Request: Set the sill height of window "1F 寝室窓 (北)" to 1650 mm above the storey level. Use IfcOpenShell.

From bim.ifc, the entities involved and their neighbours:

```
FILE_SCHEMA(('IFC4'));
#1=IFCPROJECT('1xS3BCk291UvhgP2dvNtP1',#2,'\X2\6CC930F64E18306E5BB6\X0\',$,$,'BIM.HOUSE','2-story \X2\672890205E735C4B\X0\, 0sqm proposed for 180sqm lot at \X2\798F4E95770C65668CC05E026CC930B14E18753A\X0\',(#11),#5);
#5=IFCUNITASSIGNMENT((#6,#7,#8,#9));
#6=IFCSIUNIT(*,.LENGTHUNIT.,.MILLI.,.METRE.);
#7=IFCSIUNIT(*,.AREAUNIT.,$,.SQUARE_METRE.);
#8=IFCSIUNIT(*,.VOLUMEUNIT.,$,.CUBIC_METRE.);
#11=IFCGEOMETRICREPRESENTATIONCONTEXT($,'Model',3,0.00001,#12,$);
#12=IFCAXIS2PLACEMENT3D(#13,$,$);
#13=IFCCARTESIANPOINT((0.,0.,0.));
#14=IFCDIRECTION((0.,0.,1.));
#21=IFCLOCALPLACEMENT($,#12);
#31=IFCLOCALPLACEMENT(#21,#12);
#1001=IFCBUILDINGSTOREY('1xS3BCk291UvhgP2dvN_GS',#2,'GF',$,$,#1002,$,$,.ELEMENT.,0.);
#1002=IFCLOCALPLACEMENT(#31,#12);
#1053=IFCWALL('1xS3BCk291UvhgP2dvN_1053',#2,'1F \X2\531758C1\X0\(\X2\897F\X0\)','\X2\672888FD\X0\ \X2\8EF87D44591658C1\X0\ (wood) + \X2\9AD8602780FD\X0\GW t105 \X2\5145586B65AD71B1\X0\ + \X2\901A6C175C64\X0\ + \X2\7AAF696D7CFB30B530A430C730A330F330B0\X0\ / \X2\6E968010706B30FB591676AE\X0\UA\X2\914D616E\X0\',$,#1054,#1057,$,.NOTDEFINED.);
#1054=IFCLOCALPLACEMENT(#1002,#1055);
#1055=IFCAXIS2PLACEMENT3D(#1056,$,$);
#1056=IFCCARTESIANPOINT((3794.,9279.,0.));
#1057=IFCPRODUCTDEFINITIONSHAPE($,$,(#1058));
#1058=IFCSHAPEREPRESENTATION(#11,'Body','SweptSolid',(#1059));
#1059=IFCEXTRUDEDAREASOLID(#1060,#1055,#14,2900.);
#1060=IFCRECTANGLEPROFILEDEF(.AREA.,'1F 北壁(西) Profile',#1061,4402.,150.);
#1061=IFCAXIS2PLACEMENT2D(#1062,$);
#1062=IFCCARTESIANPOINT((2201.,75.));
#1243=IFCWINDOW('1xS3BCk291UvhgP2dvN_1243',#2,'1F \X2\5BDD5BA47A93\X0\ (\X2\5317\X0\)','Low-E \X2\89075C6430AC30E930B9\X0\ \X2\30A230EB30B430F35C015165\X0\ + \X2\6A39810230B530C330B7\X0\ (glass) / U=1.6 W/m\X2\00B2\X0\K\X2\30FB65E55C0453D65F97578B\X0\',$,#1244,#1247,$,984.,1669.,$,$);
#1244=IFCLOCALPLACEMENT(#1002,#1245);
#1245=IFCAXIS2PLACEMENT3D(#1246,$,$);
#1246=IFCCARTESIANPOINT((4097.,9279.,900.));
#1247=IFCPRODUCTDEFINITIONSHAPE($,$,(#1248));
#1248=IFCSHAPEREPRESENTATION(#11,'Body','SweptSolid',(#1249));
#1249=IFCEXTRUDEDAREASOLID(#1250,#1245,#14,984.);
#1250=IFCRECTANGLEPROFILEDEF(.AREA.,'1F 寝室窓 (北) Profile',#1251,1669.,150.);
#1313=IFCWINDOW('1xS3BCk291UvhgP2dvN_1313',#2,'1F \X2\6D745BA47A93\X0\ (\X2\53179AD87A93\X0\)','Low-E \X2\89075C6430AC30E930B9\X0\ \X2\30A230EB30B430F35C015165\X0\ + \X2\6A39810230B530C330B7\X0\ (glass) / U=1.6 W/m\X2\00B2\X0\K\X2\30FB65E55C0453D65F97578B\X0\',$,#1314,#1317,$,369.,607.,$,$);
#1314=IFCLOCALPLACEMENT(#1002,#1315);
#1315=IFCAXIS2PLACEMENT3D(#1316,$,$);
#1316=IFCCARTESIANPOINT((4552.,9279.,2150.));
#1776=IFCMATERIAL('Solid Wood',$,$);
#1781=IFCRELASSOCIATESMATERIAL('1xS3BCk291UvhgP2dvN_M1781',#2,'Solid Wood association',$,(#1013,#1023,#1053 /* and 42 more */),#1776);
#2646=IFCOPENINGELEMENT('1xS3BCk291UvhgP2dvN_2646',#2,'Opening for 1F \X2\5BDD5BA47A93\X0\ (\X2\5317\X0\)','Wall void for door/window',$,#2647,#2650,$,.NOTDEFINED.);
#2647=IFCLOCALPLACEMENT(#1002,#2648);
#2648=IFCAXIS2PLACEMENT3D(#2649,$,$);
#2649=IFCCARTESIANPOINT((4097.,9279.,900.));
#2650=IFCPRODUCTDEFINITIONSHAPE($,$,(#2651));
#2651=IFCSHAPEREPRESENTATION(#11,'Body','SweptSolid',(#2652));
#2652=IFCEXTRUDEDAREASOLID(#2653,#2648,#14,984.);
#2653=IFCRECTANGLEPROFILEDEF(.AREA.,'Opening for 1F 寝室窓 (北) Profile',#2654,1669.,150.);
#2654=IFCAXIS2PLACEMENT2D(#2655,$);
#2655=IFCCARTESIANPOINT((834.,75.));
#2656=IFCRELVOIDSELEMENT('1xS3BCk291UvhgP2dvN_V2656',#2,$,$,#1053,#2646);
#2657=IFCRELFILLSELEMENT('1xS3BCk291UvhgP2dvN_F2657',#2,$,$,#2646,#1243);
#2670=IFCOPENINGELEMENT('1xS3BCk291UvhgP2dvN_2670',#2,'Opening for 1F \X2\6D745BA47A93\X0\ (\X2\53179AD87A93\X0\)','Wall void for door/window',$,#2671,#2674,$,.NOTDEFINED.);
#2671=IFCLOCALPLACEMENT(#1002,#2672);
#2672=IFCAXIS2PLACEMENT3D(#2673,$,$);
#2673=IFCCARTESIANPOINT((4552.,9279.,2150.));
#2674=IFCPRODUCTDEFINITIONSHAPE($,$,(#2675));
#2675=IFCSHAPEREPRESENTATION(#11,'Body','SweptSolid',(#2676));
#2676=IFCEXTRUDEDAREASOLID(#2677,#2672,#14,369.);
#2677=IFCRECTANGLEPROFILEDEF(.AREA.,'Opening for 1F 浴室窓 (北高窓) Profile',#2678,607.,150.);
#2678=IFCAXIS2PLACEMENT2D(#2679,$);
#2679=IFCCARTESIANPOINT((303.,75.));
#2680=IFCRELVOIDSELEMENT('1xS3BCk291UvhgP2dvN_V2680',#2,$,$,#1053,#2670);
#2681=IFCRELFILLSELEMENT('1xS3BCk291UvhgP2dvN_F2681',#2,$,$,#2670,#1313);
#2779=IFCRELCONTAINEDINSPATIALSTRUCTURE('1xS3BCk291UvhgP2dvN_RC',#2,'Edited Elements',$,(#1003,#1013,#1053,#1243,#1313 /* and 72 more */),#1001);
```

```python
import numpy as np
import ifcopenshell
import ifcopenshell.api.geometry
import ifcopenshell.geom
import ifcopenshell.util.element
import ifcopenshell.util.placement
import ifcopenshell.util.shape
import ifcopenshell.util.unit

model = ifcopenshell.open("bim.ifc")
unit_scale = ifcopenshell.util.unit.calculate_unit_scale(model)

window = model.by_guid("1xS3BCk291UvhgP2dvN_1243")
opening = window.FillsVoids[0].RelatingOpeningElement
storey = ifcopenshell.util.element.get_container(window, ifc_class="IfcBuildingStorey")
level = ifcopenshell.util.placement.get_local_placement(storey.ObjectPlacement)[2, 3]

# The opening's origin need not be at the sill, so measure its lowest point.
shape = ifcopenshell.geom.create_shape(ifcopenshell.geom.settings(), opening)
bottom = ifcopenshell.util.shape.get_shape_bottom_elevation(shape, shape.geometry) / unit_scale
dz = level + 1.65 / unit_scale - bottom

shift = np.array([0.0, 0.0, dz])
# The window is not placed relative to its opening, so move both.
for product in (opening, window):
    matrix = ifcopenshell.util.placement.get_local_placement(product.ObjectPlacement)
    matrix[:3, 3] += shift
    ifcopenshell.api.geometry.edit_object_placement(model, product=product, matrix=matrix, is_si=False)

print(f"moved by {dz * unit_scale:+.3f} m")

model.write("bim-out.ifc")
```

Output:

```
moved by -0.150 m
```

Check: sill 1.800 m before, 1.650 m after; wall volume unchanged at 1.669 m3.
